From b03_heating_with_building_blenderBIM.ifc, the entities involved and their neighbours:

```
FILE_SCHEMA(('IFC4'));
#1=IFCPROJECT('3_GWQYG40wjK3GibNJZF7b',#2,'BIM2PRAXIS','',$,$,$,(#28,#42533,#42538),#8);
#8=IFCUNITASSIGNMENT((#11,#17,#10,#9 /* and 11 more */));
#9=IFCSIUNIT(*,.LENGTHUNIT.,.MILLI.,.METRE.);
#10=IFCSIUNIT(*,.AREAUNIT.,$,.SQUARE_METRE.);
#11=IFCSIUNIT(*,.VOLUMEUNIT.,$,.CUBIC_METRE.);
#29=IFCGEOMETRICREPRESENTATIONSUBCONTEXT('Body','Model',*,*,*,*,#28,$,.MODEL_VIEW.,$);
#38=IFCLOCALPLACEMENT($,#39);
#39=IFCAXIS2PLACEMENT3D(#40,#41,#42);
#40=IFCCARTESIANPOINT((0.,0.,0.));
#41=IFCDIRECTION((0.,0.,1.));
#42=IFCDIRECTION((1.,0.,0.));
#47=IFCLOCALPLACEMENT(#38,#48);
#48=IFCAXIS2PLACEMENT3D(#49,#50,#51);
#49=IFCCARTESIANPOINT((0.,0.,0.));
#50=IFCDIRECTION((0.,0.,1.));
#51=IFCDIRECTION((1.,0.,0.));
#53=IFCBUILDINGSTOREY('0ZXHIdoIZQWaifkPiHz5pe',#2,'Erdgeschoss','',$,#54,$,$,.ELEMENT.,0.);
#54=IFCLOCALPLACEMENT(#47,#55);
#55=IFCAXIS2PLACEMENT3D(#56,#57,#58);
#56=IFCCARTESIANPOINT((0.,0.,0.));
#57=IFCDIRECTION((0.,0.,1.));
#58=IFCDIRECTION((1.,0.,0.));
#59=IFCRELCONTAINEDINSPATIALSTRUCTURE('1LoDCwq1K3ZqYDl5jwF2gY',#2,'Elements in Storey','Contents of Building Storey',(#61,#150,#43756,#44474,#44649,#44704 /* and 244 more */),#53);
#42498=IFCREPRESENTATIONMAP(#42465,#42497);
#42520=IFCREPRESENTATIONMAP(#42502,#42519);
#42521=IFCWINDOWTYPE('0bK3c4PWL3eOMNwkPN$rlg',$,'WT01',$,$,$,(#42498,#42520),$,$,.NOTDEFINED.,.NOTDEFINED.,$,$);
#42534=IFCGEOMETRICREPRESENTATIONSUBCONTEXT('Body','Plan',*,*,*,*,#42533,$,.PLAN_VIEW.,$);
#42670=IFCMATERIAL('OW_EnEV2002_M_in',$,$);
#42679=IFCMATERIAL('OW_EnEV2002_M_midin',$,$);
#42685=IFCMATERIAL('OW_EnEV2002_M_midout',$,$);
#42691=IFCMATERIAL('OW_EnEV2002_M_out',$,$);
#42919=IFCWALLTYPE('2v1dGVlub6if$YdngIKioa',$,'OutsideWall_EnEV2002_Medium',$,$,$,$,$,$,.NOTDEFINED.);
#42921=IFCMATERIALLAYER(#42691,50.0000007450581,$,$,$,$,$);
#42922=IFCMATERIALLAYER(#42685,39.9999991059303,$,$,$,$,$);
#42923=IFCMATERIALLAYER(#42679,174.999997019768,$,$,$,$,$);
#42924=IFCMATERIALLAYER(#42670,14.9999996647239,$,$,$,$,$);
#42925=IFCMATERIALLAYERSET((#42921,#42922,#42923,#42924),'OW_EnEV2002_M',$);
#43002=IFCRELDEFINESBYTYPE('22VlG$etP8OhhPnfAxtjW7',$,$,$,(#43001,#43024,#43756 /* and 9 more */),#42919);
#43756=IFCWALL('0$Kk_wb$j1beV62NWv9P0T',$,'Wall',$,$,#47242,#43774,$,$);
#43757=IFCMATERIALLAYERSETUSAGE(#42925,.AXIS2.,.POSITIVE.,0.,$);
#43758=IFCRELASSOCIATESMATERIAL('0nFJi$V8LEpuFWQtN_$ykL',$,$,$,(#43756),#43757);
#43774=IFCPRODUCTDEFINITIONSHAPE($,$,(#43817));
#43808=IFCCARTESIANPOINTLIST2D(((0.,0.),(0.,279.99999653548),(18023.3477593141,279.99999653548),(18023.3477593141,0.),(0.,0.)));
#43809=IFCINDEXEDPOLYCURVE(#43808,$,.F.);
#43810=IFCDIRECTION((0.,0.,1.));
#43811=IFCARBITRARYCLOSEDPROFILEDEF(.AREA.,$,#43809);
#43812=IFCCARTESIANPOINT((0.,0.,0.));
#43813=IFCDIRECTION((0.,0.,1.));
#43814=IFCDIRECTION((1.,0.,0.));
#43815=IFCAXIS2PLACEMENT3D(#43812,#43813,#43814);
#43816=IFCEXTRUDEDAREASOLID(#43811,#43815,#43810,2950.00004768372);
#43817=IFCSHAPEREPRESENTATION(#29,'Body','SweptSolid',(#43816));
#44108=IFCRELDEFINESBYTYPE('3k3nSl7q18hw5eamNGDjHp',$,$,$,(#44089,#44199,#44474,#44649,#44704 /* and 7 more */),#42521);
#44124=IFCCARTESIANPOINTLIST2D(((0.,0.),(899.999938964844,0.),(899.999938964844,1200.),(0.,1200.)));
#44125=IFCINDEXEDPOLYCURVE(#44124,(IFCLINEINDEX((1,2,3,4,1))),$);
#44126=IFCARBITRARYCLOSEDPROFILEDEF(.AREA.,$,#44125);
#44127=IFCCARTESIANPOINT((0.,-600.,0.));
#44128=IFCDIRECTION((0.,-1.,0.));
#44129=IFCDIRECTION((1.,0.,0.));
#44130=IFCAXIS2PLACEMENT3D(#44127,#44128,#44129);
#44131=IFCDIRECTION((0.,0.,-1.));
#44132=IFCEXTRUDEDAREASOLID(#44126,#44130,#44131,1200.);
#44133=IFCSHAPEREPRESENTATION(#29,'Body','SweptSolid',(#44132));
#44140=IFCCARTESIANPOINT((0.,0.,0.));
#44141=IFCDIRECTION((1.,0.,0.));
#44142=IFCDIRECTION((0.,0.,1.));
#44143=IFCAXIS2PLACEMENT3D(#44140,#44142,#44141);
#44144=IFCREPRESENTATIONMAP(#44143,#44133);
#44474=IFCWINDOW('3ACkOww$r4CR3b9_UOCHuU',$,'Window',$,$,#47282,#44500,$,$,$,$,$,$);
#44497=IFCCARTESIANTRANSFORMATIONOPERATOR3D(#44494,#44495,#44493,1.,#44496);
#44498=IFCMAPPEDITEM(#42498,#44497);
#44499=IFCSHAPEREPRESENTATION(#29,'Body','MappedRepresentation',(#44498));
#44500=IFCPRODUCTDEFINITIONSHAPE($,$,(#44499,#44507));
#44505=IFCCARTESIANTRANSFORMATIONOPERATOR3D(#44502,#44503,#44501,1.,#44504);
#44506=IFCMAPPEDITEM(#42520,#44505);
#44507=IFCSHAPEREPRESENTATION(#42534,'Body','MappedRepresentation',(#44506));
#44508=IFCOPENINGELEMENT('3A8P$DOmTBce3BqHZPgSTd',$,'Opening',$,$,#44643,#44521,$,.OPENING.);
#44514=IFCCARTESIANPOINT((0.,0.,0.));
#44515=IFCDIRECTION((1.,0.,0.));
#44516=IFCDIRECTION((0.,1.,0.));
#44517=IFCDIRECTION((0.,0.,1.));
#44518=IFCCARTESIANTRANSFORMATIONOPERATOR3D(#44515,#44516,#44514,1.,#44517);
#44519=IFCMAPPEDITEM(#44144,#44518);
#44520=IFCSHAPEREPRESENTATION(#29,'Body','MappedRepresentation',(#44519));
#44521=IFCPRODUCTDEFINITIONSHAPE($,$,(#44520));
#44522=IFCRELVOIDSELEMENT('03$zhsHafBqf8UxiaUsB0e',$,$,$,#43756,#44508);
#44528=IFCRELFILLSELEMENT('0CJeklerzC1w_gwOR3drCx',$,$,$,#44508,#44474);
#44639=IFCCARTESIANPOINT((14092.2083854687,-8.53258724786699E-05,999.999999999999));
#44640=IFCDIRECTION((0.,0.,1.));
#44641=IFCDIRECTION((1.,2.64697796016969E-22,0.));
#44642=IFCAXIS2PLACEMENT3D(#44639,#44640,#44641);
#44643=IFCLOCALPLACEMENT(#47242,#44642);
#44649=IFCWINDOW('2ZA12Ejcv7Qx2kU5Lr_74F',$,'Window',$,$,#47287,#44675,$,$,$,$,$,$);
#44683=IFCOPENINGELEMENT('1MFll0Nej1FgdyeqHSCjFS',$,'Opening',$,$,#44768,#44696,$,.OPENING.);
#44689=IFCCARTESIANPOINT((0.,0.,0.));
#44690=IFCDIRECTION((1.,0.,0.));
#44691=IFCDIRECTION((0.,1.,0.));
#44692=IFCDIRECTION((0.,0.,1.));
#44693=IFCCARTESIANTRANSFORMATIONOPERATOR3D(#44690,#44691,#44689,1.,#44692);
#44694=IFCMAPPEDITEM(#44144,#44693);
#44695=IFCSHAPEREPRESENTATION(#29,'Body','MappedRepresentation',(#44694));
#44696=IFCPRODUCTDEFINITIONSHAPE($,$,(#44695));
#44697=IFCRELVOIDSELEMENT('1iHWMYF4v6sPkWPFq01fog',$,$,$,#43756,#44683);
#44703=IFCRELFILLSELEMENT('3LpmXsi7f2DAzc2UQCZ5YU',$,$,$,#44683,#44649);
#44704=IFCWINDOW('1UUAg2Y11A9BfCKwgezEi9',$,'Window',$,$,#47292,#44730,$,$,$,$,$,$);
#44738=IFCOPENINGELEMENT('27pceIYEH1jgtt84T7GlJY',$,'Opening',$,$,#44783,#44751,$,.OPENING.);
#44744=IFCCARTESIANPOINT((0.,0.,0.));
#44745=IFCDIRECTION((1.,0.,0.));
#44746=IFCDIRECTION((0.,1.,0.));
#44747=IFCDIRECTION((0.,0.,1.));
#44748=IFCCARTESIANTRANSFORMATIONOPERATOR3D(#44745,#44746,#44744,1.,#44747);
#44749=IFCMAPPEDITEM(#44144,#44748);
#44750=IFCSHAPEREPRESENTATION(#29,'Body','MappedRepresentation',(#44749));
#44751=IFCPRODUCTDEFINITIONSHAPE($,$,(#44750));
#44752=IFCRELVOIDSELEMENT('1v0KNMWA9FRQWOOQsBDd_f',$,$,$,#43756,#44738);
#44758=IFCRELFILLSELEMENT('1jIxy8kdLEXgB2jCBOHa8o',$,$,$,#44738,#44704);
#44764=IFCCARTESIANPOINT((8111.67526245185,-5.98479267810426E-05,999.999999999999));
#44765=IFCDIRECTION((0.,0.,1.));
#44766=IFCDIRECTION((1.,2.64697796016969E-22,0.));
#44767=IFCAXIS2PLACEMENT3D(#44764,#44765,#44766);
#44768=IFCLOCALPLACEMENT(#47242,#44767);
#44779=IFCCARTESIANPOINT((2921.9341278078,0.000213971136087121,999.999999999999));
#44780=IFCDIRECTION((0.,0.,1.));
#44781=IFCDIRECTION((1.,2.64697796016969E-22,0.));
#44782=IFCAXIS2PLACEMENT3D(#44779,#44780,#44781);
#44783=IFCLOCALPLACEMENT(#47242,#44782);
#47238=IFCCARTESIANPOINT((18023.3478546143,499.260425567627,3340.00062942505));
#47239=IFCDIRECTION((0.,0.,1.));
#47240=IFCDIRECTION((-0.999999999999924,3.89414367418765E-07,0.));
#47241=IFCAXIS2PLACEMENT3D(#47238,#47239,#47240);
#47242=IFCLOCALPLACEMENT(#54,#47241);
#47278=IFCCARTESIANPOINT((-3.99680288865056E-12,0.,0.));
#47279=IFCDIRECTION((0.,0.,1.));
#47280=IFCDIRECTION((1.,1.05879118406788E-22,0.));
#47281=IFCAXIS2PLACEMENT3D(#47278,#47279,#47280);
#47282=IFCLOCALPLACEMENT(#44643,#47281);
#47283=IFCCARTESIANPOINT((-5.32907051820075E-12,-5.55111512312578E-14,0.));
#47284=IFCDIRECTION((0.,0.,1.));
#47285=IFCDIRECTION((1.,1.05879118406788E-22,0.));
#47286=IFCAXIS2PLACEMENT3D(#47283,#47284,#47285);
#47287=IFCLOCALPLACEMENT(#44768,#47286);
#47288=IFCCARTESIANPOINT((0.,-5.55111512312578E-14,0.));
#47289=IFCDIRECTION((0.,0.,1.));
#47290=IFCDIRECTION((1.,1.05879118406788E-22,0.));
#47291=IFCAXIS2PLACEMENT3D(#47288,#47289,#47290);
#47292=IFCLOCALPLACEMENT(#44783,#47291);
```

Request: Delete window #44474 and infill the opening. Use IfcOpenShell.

```python
import ifcopenshell
import ifcopenshell.api.feature
import ifcopenshell.api.root
import ifcopenshell.geom
import ifcopenshell.util.shape

model = ifcopenshell.open("b03_heating_with_building_blenderBIM.ifc")
settings = ifcopenshell.geom.settings()


def volume(element):
    """Net volume in cubic metres, openings subtracted."""
    shape = ifcopenshell.geom.create_shape(settings, element)
    return ifcopenshell.util.shape.get_volume(shape.geometry)


window = model.by_guid("3ACkOww$r4CR3b9_UOCHuU")
opening = window.FillsVoids[0].RelatingOpeningElement
wall = opening.VoidsElements[0].RelatingBuildingElement
before = volume(wall)

ifcopenshell.api.root.remove_product(model, product=window)
ifcopenshell.api.feature.remove_feature(model, feature=opening)

after = volume(wall)

print(f"wall volume {before:.3f} -> {after:.3f} m3")

model.write("b03_heating_with_building_blenderBIM_edited.ifc")
```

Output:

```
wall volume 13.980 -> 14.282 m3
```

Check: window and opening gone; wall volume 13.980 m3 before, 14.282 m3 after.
